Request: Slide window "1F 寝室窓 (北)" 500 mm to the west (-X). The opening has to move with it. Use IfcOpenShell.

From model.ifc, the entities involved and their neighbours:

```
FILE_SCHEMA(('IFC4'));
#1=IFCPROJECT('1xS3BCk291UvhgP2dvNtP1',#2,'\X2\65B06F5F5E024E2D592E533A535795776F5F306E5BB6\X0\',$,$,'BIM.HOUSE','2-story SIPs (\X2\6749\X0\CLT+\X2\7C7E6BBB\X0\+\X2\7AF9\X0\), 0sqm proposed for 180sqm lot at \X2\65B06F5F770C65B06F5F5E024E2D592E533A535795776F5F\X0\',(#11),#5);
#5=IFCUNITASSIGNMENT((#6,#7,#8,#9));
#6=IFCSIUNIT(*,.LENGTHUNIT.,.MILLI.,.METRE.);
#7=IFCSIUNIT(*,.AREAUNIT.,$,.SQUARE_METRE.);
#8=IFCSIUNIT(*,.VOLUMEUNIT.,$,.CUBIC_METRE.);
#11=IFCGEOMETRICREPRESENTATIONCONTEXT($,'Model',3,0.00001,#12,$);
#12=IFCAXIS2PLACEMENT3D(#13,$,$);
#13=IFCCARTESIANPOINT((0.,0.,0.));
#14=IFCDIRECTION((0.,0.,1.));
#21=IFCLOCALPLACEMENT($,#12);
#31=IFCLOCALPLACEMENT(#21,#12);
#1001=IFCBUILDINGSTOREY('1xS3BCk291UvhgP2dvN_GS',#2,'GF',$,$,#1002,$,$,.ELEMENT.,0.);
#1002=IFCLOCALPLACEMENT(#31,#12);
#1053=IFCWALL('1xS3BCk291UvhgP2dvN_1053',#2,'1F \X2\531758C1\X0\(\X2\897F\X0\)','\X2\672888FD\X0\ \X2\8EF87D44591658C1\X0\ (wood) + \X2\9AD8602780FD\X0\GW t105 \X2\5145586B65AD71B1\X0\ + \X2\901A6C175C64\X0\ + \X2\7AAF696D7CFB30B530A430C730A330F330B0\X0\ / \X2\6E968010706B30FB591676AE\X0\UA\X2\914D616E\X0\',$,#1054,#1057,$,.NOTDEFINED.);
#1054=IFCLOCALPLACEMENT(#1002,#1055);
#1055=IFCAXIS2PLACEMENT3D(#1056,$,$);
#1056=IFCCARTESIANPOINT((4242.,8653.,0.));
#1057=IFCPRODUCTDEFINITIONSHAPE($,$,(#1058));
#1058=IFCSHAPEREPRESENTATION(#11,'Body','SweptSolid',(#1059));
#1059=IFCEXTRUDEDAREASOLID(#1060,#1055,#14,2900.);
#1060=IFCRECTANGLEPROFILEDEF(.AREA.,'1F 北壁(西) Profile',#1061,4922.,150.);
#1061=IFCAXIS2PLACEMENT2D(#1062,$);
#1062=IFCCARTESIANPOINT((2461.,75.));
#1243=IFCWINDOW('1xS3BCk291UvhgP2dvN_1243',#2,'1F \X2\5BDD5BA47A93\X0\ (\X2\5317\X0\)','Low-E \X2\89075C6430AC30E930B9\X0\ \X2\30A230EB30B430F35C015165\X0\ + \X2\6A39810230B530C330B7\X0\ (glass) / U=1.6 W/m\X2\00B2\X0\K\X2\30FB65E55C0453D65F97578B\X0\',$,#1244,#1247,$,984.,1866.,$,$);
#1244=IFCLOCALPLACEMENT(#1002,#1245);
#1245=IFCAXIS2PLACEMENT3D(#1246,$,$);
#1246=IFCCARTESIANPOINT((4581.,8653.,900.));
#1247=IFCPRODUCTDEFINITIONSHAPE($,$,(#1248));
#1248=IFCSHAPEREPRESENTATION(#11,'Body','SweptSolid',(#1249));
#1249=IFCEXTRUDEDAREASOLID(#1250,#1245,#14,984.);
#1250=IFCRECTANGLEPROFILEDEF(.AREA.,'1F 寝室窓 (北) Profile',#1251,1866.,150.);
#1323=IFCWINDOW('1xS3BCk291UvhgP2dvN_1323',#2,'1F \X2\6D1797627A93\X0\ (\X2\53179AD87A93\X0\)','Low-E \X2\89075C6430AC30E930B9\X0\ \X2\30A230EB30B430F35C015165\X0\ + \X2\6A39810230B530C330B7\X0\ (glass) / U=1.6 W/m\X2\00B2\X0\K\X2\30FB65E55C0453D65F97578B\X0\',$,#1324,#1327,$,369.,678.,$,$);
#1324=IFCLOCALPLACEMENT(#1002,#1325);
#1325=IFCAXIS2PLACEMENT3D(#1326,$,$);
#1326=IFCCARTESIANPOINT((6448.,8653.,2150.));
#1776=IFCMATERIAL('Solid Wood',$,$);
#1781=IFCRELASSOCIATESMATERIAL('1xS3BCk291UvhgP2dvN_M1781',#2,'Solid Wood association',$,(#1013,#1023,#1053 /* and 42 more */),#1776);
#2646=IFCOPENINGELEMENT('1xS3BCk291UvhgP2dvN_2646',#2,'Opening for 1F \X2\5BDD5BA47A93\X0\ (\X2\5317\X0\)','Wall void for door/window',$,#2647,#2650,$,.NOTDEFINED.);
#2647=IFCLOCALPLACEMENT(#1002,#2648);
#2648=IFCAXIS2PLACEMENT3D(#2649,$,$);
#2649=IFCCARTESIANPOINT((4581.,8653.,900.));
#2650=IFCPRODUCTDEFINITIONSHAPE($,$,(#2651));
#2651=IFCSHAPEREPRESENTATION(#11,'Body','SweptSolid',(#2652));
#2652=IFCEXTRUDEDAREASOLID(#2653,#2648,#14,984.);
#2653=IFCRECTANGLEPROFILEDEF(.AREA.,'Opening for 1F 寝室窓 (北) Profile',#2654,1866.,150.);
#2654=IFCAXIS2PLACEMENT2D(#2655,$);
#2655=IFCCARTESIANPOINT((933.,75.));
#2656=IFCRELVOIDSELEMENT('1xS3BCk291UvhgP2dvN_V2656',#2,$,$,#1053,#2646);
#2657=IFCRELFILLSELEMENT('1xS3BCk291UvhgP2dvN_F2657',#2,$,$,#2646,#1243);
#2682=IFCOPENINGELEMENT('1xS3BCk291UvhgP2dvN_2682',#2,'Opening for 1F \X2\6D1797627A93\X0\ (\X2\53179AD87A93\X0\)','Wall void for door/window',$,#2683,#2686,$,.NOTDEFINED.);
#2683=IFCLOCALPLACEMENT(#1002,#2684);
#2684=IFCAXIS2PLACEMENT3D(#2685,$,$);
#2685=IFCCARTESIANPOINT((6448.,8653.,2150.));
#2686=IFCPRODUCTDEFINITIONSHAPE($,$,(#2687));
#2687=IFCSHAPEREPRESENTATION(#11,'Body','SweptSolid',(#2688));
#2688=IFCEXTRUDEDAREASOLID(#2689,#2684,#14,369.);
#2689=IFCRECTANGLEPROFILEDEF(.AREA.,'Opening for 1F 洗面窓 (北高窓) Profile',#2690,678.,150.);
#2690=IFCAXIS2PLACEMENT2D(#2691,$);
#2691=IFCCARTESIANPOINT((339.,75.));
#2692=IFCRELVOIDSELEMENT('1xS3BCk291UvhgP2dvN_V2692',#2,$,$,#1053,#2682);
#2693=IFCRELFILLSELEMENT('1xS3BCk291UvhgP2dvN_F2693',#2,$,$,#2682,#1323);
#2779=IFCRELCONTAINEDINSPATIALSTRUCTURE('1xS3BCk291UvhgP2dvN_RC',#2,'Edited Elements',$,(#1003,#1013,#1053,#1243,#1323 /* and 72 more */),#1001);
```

```python
import ifcopenshell
import ifcopenshell.api.geometry
import ifcopenshell.util.placement
import ifcopenshell.util.unit

model = ifcopenshell.open("model.ifc")
unit_scale = ifcopenshell.util.unit.calculate_unit_scale(model)

window = model.by_guid("1xS3BCk291UvhgP2dvN_1243")
opening = window.FillsVoids[0].RelatingOpeningElement
wall = opening.VoidsElements[0].RelatingBuildingElement

wall_matrix = ifcopenshell.util.placement.get_local_placement(wall.ObjectPlacement)
shift = wall_matrix[:3, 0] * -0.5 / unit_scale
before = ifcopenshell.util.placement.get_local_placement(window.ObjectPlacement)[:3, 3].copy()

# The window is not placed relative to its opening, so move both.
for product in (opening, window):
    matrix = ifcopenshell.util.placement.get_local_placement(product.ObjectPlacement)
    matrix[:3, 3] += shift
    ifcopenshell.api.geometry.edit_object_placement(model, product=product, matrix=matrix, is_si=False)

after = ifcopenshell.util.placement.get_local_placement(window.ObjectPlacement)[:3, 3]
print("window moved by", (after - before).round(3) + 0.0)

model.write("model_v2.ifc")
```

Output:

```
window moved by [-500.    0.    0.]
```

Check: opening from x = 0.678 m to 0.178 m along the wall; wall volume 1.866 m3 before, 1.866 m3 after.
